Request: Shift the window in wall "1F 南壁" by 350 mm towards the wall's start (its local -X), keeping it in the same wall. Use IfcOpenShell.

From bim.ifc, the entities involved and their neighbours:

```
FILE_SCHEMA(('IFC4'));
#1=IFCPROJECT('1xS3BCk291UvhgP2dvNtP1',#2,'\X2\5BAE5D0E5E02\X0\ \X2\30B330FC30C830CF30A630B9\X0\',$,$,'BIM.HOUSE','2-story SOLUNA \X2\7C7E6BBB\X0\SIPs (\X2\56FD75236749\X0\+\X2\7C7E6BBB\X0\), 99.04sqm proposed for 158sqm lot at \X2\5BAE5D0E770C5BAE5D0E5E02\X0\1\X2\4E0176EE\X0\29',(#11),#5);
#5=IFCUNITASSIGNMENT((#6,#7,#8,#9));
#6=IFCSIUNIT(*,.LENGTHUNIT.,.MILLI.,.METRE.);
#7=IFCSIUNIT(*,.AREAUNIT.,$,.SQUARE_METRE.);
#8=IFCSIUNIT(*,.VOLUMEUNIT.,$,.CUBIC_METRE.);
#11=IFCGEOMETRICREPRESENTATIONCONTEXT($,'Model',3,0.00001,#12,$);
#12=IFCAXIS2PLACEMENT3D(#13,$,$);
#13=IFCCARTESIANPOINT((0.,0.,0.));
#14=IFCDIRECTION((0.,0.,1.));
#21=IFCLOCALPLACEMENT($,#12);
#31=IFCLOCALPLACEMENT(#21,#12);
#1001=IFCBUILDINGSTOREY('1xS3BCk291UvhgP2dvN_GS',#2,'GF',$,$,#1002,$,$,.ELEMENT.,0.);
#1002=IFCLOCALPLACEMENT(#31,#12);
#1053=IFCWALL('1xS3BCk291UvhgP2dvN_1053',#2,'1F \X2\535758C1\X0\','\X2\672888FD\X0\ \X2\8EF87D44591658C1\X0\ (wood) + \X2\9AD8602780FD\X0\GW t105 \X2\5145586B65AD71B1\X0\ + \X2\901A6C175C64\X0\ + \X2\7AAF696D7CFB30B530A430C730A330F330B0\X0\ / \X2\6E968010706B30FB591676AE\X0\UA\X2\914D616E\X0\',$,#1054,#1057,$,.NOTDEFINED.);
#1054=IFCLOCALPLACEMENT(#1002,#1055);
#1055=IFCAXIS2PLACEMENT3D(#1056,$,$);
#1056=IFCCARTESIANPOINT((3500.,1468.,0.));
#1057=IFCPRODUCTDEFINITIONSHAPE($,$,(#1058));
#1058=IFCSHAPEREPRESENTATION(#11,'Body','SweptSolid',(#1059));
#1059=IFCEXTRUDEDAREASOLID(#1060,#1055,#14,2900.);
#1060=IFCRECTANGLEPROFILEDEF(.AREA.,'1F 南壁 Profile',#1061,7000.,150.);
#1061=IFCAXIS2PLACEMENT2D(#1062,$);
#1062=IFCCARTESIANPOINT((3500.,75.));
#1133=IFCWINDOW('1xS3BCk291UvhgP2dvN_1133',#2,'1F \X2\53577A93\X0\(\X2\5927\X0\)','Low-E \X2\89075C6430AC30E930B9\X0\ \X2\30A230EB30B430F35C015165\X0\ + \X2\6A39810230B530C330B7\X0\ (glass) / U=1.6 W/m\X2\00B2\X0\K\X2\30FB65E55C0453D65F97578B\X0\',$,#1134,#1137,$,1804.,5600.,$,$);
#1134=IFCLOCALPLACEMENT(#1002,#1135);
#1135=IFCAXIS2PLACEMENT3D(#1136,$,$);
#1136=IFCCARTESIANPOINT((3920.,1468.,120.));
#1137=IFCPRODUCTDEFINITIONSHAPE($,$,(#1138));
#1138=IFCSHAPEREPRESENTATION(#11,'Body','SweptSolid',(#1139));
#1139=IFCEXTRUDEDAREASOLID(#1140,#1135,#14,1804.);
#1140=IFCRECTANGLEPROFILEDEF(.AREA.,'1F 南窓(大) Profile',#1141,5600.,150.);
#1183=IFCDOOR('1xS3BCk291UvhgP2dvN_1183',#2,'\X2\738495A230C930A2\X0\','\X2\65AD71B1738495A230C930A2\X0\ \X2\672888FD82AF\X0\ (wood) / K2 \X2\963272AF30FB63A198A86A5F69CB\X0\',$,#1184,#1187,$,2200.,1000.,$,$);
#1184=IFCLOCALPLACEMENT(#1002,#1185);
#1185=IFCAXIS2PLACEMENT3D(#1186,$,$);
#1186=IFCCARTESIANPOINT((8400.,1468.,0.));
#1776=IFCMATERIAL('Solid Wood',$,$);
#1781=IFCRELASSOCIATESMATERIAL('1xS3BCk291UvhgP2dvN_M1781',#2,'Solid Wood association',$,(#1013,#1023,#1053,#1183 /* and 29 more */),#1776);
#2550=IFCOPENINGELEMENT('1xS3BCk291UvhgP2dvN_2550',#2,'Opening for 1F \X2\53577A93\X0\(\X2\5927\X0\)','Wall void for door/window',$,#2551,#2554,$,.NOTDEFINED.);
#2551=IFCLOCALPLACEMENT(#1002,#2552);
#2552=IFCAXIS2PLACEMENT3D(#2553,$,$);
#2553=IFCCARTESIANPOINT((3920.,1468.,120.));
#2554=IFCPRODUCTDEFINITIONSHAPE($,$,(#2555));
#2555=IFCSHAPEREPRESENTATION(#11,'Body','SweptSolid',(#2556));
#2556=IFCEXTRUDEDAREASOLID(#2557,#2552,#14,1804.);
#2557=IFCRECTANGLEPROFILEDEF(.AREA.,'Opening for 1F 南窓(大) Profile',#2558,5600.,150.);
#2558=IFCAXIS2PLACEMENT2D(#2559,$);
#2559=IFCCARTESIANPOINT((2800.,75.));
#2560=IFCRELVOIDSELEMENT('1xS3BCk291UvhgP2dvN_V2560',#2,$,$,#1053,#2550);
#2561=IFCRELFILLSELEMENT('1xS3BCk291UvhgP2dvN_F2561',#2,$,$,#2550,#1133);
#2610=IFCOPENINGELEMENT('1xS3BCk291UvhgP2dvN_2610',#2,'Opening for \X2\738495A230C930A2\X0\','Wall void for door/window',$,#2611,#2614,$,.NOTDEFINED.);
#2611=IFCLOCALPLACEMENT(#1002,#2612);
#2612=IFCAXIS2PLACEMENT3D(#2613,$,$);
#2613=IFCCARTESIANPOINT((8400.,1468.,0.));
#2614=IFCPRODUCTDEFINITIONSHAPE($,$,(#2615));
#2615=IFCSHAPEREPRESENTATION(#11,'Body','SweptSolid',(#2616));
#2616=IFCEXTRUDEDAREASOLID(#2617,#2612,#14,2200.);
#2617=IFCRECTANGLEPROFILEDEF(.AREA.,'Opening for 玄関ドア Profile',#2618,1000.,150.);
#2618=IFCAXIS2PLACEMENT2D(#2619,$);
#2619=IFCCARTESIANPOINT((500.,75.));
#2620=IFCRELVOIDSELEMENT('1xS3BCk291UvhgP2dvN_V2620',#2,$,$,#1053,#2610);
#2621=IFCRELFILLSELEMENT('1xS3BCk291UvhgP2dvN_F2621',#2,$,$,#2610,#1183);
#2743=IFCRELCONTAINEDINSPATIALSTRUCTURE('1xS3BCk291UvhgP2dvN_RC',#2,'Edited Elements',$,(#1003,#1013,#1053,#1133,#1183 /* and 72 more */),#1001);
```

```python
import ifcopenshell
import ifcopenshell.api.geometry
import ifcopenshell.util.placement
import ifcopenshell.util.unit

model = ifcopenshell.open("bim.ifc")
unit_scale = ifcopenshell.util.unit.calculate_unit_scale(model)

window = model.by_guid("1xS3BCk291UvhgP2dvN_1133")
opening = window.FillsVoids[0].RelatingOpeningElement
wall = opening.VoidsElements[0].RelatingBuildingElement

wall_matrix = ifcopenshell.util.placement.get_local_placement(wall.ObjectPlacement)
shift = wall_matrix[:3, 0] * -0.35 / unit_scale
before = ifcopenshell.util.placement.get_local_placement(window.ObjectPlacement)[:3, 3].copy()

# The window is not placed relative to its opening, so move both.
for product in (opening, window):
    matrix = ifcopenshell.util.placement.get_local_placement(product.ObjectPlacement)
    matrix[:3, 3] += shift
    ifcopenshell.api.geometry.edit_object_placement(model, product=product, matrix=matrix, is_si=False)

after = ifcopenshell.util.placement.get_local_placement(window.ObjectPlacement)[:3, 3]
print("window moved by", (after - before).round(3) + 0.0)

model.write("bim_rev.ifc")
```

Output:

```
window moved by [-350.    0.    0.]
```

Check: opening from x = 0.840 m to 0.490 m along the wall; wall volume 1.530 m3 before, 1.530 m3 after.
